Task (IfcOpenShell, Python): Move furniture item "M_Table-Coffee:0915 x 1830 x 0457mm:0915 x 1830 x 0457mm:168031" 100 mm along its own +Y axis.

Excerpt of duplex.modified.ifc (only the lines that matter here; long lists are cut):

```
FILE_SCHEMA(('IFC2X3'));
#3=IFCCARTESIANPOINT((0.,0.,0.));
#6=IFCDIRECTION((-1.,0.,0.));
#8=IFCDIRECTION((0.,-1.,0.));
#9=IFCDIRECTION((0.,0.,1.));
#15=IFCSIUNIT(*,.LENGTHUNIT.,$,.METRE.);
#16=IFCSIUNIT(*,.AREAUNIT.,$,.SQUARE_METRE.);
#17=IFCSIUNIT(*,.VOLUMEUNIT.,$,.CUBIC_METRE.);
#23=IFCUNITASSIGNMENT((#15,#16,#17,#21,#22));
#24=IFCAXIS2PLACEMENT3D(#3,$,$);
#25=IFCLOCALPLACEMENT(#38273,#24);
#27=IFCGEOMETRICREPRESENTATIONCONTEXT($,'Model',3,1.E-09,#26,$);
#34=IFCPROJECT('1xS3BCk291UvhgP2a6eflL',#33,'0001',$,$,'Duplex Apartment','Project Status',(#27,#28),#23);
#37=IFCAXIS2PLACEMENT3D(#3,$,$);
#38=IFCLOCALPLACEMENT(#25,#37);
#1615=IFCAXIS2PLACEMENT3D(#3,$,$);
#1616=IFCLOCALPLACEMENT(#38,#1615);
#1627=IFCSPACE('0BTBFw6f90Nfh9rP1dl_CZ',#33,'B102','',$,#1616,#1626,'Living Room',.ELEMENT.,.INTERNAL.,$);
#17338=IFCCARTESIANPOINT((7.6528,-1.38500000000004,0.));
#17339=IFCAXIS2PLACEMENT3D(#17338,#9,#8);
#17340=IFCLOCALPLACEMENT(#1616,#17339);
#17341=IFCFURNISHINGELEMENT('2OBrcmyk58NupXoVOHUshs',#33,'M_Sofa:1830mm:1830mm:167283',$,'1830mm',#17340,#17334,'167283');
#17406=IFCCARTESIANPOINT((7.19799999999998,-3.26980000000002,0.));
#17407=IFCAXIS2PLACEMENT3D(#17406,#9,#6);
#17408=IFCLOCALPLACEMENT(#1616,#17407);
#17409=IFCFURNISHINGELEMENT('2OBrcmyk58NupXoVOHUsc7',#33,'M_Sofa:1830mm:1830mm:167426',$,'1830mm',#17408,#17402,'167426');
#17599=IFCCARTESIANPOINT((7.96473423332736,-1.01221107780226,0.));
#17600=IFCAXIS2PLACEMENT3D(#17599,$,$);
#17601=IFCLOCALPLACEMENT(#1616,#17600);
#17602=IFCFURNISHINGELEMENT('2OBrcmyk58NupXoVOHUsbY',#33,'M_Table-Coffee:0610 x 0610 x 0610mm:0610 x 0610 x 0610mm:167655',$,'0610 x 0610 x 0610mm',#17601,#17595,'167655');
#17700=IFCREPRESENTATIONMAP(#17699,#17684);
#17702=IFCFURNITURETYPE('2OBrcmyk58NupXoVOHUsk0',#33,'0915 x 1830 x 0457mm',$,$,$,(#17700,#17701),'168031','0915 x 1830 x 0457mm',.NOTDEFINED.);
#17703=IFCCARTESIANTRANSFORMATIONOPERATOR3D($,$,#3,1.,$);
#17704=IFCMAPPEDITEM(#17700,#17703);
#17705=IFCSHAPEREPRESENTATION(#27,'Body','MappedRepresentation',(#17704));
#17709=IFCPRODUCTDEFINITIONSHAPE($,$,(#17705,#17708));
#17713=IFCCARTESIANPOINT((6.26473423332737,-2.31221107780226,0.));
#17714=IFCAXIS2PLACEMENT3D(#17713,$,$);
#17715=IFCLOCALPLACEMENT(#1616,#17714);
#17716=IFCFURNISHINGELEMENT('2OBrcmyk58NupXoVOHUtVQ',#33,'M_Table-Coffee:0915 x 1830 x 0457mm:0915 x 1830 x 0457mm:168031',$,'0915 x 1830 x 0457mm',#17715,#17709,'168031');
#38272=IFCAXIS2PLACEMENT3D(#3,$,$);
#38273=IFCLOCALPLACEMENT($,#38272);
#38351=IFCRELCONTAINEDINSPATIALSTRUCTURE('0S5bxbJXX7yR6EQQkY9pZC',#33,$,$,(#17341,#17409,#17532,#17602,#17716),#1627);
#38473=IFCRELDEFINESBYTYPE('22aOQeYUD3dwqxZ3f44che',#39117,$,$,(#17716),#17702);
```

```python
import ifcopenshell
import ifcopenshell.api.geometry
import ifcopenshell.util.placement
import ifcopenshell.util.unit

model = ifcopenshell.open("duplex.modified.ifc")
unit_scale = ifcopenshell.util.unit.calculate_unit_scale(model)

item = model.by_guid("2OBrcmyk58NupXoVOHUtVQ")
matrix = ifcopenshell.util.placement.get_local_placement(item.ObjectPlacement)
matrix[:3, 3] += matrix[:3, 1] * 0.1 / unit_scale
ifcopenshell.api.geometry.edit_object_placement(model, product=item, matrix=matrix, is_si=False)

print(ifcopenshell.util.placement.get_local_placement(item.ObjectPlacement).round(3) + 0.0)

model.write("duplex.modified_updated.ifc")
```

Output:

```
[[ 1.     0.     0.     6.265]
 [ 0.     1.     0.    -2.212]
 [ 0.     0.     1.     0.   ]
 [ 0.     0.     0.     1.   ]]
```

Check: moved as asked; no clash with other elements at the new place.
